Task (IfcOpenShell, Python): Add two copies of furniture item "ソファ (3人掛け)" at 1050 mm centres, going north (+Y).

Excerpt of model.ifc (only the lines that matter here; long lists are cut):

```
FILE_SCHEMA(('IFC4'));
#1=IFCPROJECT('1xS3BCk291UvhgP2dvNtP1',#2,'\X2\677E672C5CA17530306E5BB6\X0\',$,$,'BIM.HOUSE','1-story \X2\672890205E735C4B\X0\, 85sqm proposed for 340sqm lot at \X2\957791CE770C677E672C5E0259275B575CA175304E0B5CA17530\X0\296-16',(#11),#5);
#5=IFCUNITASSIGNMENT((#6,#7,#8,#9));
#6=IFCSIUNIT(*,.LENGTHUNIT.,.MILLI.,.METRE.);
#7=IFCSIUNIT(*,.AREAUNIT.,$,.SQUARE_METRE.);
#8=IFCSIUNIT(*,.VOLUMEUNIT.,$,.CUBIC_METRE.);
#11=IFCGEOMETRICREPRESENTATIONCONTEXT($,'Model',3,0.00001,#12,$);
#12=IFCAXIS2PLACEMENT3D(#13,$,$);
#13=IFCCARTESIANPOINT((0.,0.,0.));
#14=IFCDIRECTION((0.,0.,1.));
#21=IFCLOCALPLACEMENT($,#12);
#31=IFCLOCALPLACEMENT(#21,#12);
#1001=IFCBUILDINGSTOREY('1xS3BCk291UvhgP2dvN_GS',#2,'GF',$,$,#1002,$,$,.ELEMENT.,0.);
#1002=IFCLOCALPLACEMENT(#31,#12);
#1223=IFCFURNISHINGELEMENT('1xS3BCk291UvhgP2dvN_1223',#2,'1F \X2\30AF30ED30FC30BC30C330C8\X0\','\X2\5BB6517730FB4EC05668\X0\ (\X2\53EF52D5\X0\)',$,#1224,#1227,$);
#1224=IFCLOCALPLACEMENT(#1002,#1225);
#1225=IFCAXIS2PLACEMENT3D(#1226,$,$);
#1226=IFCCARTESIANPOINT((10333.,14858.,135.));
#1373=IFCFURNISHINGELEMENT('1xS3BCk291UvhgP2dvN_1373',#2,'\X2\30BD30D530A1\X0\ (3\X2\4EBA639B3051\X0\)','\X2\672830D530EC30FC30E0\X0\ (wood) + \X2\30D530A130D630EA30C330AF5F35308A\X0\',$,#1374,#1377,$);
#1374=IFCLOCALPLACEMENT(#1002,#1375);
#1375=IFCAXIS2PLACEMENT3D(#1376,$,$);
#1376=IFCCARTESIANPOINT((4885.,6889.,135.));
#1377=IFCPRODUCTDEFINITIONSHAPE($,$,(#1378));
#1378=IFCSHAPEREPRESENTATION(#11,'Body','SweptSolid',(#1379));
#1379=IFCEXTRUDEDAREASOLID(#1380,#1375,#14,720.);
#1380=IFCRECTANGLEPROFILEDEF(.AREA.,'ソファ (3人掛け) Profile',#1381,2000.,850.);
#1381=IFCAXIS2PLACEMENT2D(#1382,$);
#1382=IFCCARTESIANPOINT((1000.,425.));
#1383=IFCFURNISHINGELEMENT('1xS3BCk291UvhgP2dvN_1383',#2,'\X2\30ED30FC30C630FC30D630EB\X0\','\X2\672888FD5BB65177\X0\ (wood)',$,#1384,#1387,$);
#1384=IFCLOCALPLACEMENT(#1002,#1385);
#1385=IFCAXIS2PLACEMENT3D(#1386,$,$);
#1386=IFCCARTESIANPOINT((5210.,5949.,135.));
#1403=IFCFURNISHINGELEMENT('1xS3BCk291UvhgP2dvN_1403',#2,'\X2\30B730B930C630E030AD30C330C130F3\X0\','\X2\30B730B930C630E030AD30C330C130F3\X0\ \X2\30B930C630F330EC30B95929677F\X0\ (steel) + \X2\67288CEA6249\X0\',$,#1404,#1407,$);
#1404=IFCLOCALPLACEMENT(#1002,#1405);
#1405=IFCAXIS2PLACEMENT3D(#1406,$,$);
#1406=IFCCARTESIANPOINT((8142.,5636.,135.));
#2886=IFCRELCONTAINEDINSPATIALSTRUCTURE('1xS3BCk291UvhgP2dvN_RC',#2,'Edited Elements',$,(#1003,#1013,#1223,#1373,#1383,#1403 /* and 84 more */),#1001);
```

```python
import numpy as np
import ifcopenshell
import ifcopenshell.api.geometry
import ifcopenshell.api.root
import ifcopenshell.util.element
import ifcopenshell.util.placement
import ifcopenshell.util.unit

model = ifcopenshell.open("model.ifc")
unit_scale = ifcopenshell.util.unit.calculate_unit_scale(model)


def reuse_history(source, copy):
    """copy_class also copies each property set's owner history, people and application; keep the originals."""
    for rel in copy.IsDefinedBy:
        if rel.is_a("IfcRelDefinesByProperties") and (history := rel.RelatingPropertyDefinition.OwnerHistory):
            rel.RelatingPropertyDefinition.OwnerHistory = source.OwnerHistory
            ifcopenshell.util.element.remove_deep2(model, history)


source = model.by_guid("1xS3BCk291UvhgP2dvN_1373")
base = ifcopenshell.util.placement.get_local_placement(source.ObjectPlacement)
step = np.array([0.0, 1.0, 0.0]) * 1.05 / unit_scale

for i in range(1, 3):
    copy = ifcopenshell.api.root.copy_class(model, product=source)
    copy.Representation = ifcopenshell.util.element.copy_deep(
        model, source.Representation, exclude=["IfcGeometricRepresentationContext", "IfcRepresentationMap"]
    )
    reuse_history(source, copy)
    matrix = base.copy()
    matrix[:3, 3] += i * step
    print("added at", matrix[:3, 3].round(3) + 0.0)
    ifcopenshell.api.geometry.edit_object_placement(model, product=copy, matrix=matrix, is_si=False)

model.write("model_updated.ifc")
```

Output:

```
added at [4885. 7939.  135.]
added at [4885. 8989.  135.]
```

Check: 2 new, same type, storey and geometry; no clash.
